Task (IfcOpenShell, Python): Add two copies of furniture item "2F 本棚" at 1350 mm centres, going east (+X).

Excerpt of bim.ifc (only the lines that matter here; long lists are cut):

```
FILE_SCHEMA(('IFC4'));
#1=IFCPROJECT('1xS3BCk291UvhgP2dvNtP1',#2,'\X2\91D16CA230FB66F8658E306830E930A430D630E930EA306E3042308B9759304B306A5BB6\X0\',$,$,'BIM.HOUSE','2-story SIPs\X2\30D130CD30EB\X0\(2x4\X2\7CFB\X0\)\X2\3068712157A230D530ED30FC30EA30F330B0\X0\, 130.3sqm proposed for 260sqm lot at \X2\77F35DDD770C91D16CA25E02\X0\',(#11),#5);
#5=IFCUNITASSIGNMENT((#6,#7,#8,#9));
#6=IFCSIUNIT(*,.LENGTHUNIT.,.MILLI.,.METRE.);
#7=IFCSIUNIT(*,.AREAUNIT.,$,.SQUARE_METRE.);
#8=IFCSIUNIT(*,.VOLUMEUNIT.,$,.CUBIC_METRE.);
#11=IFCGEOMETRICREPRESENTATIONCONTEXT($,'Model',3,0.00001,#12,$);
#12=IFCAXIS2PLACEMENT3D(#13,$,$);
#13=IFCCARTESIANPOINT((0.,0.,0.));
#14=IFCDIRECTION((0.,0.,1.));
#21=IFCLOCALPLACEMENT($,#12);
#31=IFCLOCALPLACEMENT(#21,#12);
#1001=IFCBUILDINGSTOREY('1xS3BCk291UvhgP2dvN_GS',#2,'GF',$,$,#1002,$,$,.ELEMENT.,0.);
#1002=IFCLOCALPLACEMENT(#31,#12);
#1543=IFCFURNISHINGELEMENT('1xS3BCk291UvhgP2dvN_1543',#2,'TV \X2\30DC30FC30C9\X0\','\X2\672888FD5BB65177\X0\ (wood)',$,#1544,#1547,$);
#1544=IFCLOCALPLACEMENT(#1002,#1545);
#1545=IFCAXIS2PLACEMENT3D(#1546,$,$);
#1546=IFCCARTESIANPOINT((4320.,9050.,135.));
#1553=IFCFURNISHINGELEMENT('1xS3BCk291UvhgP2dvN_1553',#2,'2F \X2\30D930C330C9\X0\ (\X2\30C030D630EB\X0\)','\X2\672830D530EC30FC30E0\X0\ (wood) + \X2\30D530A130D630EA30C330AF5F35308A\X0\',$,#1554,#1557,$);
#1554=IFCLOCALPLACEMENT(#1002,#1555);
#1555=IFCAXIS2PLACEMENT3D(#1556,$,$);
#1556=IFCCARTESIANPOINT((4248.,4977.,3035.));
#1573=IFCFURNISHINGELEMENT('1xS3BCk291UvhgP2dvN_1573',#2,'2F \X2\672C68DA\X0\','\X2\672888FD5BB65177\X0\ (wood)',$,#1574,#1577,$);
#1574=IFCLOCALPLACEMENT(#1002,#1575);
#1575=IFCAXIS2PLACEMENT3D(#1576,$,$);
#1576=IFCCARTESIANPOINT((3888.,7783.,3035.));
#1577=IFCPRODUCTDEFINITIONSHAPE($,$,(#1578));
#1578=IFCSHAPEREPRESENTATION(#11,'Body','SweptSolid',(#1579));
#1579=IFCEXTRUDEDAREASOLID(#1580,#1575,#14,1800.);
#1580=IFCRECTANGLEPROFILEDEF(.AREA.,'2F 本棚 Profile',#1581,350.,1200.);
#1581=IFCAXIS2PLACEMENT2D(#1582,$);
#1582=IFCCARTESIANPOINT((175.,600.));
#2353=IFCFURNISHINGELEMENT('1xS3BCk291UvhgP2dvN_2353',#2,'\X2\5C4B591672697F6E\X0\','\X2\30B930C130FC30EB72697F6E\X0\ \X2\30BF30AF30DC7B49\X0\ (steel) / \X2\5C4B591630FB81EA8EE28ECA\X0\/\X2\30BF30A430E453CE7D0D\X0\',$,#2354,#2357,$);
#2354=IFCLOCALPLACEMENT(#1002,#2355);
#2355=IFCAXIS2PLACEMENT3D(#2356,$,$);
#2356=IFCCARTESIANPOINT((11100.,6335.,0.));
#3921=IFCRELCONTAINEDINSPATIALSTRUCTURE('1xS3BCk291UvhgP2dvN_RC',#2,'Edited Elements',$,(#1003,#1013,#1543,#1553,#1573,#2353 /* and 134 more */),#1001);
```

```python
import numpy as np
import ifcopenshell
import ifcopenshell.api.geometry
import ifcopenshell.api.root
import ifcopenshell.util.element
import ifcopenshell.util.placement
import ifcopenshell.util.unit

model = ifcopenshell.open("bim.ifc")
unit_scale = ifcopenshell.util.unit.calculate_unit_scale(model)


def reuse_history(source, copy):
    """copy_class also copies each property set's owner history, people and application; keep the originals."""
    for rel in copy.IsDefinedBy:
        if rel.is_a("IfcRelDefinesByProperties") and (history := rel.RelatingPropertyDefinition.OwnerHistory):
            rel.RelatingPropertyDefinition.OwnerHistory = source.OwnerHistory
            ifcopenshell.util.element.remove_deep2(model, history)


source = model.by_id(1573)
base = ifcopenshell.util.placement.get_local_placement(source.ObjectPlacement)
step = np.array([1.0, 0.0, 0.0]) * 1.35 / unit_scale

for i in range(1, 3):
    copy = ifcopenshell.api.root.copy_class(model, product=source)
    copy.Representation = ifcopenshell.util.element.copy_deep(
        model, source.Representation, exclude=["IfcGeometricRepresentationContext", "IfcRepresentationMap"]
    )
    reuse_history(source, copy)
    matrix = base.copy()
    matrix[:3, 3] += i * step
    print("added at", matrix[:3, 3].round(3) + 0.0)
    ifcopenshell.api.geometry.edit_object_placement(model, product=copy, matrix=matrix, is_si=False)

model.write("bim_v2.ifc")
```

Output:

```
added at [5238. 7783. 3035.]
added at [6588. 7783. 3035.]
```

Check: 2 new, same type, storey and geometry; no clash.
